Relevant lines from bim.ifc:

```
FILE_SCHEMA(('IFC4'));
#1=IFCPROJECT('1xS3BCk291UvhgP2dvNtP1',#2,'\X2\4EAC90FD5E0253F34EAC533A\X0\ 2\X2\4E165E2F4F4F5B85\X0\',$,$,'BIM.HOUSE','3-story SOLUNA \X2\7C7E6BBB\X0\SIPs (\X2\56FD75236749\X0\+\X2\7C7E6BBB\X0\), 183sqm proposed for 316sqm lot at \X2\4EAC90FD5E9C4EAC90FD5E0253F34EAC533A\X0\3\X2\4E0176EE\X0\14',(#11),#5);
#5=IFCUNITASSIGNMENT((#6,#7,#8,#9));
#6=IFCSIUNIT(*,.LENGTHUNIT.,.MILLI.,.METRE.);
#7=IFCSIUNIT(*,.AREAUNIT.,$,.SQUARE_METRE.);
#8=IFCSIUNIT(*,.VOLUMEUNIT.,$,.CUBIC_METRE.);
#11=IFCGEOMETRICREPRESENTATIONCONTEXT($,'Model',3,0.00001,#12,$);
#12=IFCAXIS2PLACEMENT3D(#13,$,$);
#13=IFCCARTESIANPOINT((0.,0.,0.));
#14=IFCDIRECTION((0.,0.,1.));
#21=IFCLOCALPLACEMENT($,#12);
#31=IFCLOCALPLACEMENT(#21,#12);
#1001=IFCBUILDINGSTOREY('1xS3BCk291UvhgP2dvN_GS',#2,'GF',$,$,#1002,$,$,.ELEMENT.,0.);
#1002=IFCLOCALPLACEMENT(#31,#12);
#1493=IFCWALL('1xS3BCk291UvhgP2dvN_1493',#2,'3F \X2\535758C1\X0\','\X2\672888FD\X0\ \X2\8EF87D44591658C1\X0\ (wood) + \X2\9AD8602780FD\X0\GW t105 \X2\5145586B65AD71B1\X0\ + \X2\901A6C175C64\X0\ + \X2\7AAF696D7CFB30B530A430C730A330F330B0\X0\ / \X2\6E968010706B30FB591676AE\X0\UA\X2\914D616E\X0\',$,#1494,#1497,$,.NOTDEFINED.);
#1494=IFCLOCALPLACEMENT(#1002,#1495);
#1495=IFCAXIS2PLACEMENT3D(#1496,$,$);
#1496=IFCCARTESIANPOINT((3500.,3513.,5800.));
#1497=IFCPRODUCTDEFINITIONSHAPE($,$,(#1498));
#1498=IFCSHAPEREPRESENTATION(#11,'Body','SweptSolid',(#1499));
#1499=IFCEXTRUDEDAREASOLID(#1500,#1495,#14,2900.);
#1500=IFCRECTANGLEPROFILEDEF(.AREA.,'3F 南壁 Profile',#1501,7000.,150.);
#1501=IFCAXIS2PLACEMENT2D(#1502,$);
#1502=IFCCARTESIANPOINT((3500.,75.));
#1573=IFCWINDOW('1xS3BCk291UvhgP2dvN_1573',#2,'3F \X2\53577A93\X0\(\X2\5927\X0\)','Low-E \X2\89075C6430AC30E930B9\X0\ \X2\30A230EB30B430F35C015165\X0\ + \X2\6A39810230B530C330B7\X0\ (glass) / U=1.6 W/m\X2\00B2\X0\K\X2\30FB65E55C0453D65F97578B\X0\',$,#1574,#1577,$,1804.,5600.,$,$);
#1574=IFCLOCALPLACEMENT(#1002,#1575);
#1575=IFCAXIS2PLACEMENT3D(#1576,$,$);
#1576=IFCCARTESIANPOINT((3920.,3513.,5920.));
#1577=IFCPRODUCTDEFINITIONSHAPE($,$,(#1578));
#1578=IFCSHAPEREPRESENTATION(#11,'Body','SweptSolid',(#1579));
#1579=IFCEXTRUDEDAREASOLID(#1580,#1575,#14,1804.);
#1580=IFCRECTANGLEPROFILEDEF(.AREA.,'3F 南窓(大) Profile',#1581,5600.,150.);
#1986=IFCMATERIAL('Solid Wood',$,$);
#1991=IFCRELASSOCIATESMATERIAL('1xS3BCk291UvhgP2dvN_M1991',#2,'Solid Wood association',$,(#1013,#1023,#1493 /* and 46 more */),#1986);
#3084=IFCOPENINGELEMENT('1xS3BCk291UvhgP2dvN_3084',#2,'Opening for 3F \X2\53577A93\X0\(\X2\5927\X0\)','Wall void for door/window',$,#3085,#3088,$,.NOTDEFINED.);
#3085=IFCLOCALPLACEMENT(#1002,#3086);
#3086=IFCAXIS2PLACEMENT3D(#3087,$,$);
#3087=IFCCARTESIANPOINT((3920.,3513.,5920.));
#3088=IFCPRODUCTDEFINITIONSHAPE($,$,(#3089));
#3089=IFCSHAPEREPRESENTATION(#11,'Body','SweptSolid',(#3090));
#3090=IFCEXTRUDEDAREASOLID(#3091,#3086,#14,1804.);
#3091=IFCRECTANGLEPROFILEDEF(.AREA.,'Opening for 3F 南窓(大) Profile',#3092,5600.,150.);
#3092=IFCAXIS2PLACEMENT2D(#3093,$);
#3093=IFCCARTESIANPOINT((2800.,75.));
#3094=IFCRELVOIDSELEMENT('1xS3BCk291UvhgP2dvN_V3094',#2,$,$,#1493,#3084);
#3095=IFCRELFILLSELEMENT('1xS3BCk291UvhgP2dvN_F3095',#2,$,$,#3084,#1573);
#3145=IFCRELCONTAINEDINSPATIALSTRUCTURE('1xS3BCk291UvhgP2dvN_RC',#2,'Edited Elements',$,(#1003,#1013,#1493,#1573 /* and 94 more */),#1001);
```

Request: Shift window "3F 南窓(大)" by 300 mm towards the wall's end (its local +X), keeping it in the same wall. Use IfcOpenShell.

```python
import ifcopenshell
import ifcopenshell.api.geometry
import ifcopenshell.util.placement

model = ifcopenshell.open("bim.ifc")

window = model.by_guid("1xS3BCk291UvhgP2dvN_1573")
opening = window.FillsVoids[0].RelatingOpeningElement
wall = opening.VoidsElements[0].RelatingBuildingElement

wall_matrix = ifcopenshell.util.placement.get_local_placement(wall.ObjectPlacement)
shift = wall_matrix[:3, 0] * 300.0
before = ifcopenshell.util.placement.get_local_placement(window.ObjectPlacement)[:3, 3].copy()

# The window is not placed relative to its opening, so move both.
for product in (opening, window):
    matrix = ifcopenshell.util.placement.get_local_placement(product.ObjectPlacement)
    matrix[:3, 3] += shift
    ifcopenshell.api.geometry.edit_object_placement(model, product=product, matrix=matrix, is_si=False)

after = ifcopenshell.util.placement.get_local_placement(window.ObjectPlacement)[:3, 3]
print("window moved by", (after - before).round(3) + 0.0)

model.write("bim_rev.ifc")
```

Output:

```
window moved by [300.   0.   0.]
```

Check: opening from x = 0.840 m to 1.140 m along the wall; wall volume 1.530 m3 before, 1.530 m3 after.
